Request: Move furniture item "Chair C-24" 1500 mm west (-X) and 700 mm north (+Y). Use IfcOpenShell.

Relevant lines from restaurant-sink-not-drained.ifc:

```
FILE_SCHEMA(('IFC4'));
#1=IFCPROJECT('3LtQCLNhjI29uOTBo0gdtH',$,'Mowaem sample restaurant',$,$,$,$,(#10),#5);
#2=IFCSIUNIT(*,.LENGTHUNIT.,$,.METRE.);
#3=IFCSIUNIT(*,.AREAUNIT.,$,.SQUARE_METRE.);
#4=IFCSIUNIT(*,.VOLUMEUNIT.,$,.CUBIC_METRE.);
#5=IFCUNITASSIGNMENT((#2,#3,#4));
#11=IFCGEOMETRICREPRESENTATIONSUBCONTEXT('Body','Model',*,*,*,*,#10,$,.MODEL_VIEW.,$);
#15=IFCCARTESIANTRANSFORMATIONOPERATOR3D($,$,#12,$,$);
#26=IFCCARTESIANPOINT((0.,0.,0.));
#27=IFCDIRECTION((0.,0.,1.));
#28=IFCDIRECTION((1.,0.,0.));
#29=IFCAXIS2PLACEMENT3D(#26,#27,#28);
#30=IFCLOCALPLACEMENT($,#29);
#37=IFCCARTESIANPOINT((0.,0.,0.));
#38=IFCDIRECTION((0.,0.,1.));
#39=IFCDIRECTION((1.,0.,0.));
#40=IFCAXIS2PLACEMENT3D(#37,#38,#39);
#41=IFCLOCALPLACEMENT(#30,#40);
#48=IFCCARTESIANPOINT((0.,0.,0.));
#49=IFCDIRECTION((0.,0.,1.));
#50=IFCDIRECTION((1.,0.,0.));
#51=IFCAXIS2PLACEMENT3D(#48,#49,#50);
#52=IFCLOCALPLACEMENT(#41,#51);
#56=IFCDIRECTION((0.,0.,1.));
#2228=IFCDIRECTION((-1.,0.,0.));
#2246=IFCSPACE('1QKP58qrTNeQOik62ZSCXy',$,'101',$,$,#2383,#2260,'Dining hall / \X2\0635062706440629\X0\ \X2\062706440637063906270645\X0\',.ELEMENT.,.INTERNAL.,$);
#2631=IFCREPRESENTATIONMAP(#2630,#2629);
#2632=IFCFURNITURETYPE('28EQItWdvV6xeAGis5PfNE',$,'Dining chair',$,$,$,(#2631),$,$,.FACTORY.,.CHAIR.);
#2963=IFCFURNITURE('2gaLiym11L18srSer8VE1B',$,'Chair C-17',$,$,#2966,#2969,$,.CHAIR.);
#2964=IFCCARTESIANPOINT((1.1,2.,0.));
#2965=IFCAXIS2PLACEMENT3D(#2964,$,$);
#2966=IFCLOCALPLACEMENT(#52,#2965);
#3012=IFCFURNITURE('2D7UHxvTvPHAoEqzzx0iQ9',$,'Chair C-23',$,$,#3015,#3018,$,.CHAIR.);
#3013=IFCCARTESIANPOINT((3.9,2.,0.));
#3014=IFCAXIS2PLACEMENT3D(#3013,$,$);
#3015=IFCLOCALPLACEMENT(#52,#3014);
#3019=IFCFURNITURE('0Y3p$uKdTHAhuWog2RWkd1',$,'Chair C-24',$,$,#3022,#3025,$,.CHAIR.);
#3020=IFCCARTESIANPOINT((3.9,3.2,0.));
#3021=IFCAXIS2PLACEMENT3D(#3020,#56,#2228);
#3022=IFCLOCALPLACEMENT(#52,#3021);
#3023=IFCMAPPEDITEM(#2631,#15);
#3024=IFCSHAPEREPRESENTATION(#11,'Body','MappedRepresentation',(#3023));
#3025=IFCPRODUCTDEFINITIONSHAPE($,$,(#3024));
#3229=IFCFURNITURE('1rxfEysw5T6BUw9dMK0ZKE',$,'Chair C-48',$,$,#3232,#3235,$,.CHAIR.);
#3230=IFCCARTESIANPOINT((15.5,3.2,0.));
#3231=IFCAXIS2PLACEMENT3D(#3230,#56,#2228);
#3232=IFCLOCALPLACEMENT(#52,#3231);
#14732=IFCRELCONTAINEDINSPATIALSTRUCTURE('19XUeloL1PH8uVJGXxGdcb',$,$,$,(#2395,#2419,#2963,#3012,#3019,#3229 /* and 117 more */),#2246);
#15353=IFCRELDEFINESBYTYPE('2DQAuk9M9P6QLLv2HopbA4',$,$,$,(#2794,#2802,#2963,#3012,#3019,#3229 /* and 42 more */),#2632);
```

```python
import ifcopenshell
import ifcopenshell.api.geometry
import ifcopenshell.util.placement

model = ifcopenshell.open("restaurant-sink-not-drained.ifc")

item = model.by_guid("0Y3p$uKdTHAhuWog2RWkd1")
matrix = ifcopenshell.util.placement.get_local_placement(item.ObjectPlacement)
matrix[0, 3] -= 1.5
matrix[1, 3] += 0.7
ifcopenshell.api.geometry.edit_object_placement(model, product=item, matrix=matrix, is_si=False)

print(ifcopenshell.util.placement.get_local_placement(item.ObjectPlacement).round(3) + 0.0)

model.write("restaurant-sink-not-drained_v2.ifc")
```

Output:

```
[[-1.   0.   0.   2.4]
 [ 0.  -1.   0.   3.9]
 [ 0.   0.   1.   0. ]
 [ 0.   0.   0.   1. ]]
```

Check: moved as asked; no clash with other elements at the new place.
